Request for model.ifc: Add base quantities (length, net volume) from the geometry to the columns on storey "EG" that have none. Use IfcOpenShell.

First a look at what the model holds.

```python
import ifcopenshell
import ifcopenshell.util.element
import ifcopenshell.util.unit

model = ifcopenshell.open("model.ifc")
print(model.schema)
for unit_type in ("LENGTHUNIT", "AREAUNIT", "VOLUMEUNIT"):
    print(unit_type, ifcopenshell.util.unit.calculate_unit_scale(model, unit_type))
storey = next(s for s in model.by_type("IfcBuildingStorey") if s.Name == "EG")
columns = [e for e in ifcopenshell.util.element.get_decomposition(storey) if e.is_a("IfcColumn")]
for e in sorted(columns, key=lambda e: e.id()):
    print(e.id(), e.is_a(), e.Name, list(ifcopenshell.util.element.get_psets(e, qtos_only=True)), sep=" | ")
```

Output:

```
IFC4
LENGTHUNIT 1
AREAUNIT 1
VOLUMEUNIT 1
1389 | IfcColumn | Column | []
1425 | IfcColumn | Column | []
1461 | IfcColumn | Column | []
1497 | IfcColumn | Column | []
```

```python
import ifcopenshell
import ifcopenshell.api.pset
import ifcopenshell.geom
import ifcopenshell.util.element
import ifcopenshell.util.shape
import ifcopenshell.util.unit

model = ifcopenshell.open("model.ifc")
unit_scale = ifcopenshell.util.unit.calculate_unit_scale(model)
volume_scale = ifcopenshell.util.unit.calculate_unit_scale(model, "VOLUMEUNIT")
settings = ifcopenshell.geom.settings()

storey = next(s for s in model.by_type("IfcBuildingStorey") if s.Name == "EG")
columns = [e for e in ifcopenshell.util.element.get_decomposition(storey) if e.is_a("IfcColumn")]

for e in sorted(columns, key=lambda e: e.id()):
    if ifcopenshell.util.element.get_psets(e, qtos_only=True, should_inherit=False):
        continue
    # Geometry comes back in metres, in the element's own axes.
    shape = ifcopenshell.geom.create_shape(settings, e)
    values = {
        "Length": ifcopenshell.util.shape.get_z(shape.geometry) / unit_scale,
        "NetVolume": ifcopenshell.util.shape.get_volume(shape.geometry) / volume_scale,
    }
    qto = ifcopenshell.api.pset.add_qto(model, product=e, name="Qto_ColumnBaseQuantities")
    ifcopenshell.api.pset.edit_qto(model, qto=qto, properties=values)
    print(e.id(), {k: round(v, 3) for k, v in values.items()})

model.write("model_edited.ifc")
```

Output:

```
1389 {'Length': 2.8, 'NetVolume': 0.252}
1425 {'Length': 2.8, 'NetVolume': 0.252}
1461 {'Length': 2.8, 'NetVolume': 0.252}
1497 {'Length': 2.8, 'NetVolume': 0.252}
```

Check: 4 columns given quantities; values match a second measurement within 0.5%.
